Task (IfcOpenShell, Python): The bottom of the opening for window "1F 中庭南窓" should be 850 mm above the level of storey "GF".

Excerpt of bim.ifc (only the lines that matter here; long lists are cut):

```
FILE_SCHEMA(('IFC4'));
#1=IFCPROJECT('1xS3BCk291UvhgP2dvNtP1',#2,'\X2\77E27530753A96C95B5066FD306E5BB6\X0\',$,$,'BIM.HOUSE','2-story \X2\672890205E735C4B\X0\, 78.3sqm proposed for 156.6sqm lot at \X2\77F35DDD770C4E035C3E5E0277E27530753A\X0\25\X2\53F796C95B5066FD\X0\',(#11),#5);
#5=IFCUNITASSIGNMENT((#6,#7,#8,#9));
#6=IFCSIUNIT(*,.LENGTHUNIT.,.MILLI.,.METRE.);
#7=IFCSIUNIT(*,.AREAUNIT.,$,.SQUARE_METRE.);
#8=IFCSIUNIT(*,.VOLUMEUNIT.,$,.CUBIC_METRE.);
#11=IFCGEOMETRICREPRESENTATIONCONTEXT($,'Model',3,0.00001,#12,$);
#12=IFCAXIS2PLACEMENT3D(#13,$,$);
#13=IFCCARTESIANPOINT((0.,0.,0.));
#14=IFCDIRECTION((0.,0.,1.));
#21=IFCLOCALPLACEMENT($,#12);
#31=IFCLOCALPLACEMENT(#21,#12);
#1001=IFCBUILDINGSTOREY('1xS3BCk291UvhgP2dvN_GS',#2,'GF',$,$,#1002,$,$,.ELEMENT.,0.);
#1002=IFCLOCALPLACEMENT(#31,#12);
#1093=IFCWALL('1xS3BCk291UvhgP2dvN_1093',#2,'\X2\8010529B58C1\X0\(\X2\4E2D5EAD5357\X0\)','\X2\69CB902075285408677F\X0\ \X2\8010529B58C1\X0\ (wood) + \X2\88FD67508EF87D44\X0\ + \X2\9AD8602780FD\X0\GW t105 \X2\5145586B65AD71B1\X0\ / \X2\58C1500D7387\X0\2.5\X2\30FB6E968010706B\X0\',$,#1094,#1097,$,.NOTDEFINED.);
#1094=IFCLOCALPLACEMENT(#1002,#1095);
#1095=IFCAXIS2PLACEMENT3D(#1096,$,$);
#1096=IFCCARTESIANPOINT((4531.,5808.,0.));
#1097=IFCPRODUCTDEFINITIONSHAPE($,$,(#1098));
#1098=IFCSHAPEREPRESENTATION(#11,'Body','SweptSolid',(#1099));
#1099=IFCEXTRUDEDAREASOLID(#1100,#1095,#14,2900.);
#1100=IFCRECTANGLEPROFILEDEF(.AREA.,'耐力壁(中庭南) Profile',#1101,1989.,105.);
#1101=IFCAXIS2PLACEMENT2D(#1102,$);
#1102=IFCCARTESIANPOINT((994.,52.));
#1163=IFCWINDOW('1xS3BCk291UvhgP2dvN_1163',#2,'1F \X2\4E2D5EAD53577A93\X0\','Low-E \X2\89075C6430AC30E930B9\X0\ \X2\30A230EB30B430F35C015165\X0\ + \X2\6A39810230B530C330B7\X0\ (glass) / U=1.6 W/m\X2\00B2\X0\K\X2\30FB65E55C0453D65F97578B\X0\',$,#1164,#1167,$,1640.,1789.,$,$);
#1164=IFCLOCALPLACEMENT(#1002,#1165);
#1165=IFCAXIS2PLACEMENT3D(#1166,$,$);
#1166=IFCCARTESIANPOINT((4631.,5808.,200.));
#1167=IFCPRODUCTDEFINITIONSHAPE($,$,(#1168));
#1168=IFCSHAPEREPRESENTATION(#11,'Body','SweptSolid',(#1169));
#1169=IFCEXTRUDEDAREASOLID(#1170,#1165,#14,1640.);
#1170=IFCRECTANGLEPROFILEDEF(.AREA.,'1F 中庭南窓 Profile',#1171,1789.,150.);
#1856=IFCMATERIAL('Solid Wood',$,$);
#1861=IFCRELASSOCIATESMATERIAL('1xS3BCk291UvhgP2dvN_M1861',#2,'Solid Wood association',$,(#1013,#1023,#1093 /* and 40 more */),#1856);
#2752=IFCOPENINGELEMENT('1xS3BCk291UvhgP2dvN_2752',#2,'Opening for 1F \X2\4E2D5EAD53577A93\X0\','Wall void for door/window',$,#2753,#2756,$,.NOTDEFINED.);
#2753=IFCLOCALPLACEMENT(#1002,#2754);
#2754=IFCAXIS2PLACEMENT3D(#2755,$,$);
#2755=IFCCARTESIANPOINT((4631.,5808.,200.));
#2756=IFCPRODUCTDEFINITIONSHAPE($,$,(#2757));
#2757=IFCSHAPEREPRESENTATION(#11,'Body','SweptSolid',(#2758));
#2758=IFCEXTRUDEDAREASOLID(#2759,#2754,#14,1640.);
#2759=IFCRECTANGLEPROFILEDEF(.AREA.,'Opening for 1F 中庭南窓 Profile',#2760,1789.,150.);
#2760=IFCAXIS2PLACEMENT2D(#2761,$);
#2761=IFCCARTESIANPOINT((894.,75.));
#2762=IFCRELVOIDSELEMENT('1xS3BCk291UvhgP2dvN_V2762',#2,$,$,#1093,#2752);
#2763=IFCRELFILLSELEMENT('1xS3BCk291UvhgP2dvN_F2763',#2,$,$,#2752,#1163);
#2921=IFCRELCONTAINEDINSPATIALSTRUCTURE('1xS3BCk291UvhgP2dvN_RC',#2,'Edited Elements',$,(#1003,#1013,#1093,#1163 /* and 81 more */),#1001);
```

```python
import numpy as np
import ifcopenshell
import ifcopenshell.api.geometry
import ifcopenshell.geom
import ifcopenshell.util.element
import ifcopenshell.util.placement
import ifcopenshell.util.shape
import ifcopenshell.util.unit

model = ifcopenshell.open("bim.ifc")
unit_scale = ifcopenshell.util.unit.calculate_unit_scale(model)

window = model.by_guid("1xS3BCk291UvhgP2dvN_1163")
opening = window.FillsVoids[0].RelatingOpeningElement
storey = ifcopenshell.util.element.get_container(window, ifc_class="IfcBuildingStorey")
level = ifcopenshell.util.placement.get_local_placement(storey.ObjectPlacement)[2, 3]

# The opening's origin need not be at the sill, so measure its lowest point.
shape = ifcopenshell.geom.create_shape(ifcopenshell.geom.settings(), opening)
bottom = ifcopenshell.util.shape.get_shape_bottom_elevation(shape, shape.geometry) / unit_scale
dz = level + 0.85 / unit_scale - bottom

shift = np.array([0.0, 0.0, dz])
# The window is not placed relative to its opening, so move both.
for product in (opening, window):
    matrix = ifcopenshell.util.placement.get_local_placement(product.ObjectPlacement)
    matrix[:3, 3] += shift
    ifcopenshell.api.geometry.edit_object_placement(model, product=product, matrix=matrix, is_si=False)

print(f"moved by {dz * unit_scale:+.3f} m")

model.write("bim_v2.ifc")
```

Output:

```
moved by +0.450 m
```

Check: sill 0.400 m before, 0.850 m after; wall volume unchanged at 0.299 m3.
